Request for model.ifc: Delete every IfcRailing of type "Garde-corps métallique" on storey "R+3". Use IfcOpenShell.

First a look at what the model holds.

```python
import ifcopenshell
import ifcopenshell.util.element

model = ifcopenshell.open("model.ifc")
print(model.schema)
storey = next(s for s in model.by_type("IfcBuildingStorey") if s.Name == "R+3")
railings = [e for e in ifcopenshell.util.element.get_decomposition(storey) if e.is_a("IfcRailing")]
seen = {}
for e in railings:
    element_type = ifcopenshell.util.element.get_type(e)
    name = element_type.Name if element_type not in (None, e) else None
    seen[name] = seen.get(name, 0) + 1
for name, count in sorted(seen.items(), key=str):
    print(count, "x", name)
```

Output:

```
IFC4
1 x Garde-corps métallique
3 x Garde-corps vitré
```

```python
import ifcopenshell
import ifcopenshell.api.root
import ifcopenshell.util.element

model = ifcopenshell.open("model.ifc")

storey = next(s for s in model.by_type("IfcBuildingStorey") if s.Name == "R+3")
railings = [e for e in ifcopenshell.util.element.get_decomposition(storey) if e.is_a("IfcRailing")]
targets = [e for e in railings if (t := ifcopenshell.util.element.get_type(e)) not in (None, e) and t.Name == "Garde-corps métallique"]

for e in targets:
    ifcopenshell.api.root.remove_product(model, product=e)
print(len(targets), "removed")

model.write("model_edited.ifc")
```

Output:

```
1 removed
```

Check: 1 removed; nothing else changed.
